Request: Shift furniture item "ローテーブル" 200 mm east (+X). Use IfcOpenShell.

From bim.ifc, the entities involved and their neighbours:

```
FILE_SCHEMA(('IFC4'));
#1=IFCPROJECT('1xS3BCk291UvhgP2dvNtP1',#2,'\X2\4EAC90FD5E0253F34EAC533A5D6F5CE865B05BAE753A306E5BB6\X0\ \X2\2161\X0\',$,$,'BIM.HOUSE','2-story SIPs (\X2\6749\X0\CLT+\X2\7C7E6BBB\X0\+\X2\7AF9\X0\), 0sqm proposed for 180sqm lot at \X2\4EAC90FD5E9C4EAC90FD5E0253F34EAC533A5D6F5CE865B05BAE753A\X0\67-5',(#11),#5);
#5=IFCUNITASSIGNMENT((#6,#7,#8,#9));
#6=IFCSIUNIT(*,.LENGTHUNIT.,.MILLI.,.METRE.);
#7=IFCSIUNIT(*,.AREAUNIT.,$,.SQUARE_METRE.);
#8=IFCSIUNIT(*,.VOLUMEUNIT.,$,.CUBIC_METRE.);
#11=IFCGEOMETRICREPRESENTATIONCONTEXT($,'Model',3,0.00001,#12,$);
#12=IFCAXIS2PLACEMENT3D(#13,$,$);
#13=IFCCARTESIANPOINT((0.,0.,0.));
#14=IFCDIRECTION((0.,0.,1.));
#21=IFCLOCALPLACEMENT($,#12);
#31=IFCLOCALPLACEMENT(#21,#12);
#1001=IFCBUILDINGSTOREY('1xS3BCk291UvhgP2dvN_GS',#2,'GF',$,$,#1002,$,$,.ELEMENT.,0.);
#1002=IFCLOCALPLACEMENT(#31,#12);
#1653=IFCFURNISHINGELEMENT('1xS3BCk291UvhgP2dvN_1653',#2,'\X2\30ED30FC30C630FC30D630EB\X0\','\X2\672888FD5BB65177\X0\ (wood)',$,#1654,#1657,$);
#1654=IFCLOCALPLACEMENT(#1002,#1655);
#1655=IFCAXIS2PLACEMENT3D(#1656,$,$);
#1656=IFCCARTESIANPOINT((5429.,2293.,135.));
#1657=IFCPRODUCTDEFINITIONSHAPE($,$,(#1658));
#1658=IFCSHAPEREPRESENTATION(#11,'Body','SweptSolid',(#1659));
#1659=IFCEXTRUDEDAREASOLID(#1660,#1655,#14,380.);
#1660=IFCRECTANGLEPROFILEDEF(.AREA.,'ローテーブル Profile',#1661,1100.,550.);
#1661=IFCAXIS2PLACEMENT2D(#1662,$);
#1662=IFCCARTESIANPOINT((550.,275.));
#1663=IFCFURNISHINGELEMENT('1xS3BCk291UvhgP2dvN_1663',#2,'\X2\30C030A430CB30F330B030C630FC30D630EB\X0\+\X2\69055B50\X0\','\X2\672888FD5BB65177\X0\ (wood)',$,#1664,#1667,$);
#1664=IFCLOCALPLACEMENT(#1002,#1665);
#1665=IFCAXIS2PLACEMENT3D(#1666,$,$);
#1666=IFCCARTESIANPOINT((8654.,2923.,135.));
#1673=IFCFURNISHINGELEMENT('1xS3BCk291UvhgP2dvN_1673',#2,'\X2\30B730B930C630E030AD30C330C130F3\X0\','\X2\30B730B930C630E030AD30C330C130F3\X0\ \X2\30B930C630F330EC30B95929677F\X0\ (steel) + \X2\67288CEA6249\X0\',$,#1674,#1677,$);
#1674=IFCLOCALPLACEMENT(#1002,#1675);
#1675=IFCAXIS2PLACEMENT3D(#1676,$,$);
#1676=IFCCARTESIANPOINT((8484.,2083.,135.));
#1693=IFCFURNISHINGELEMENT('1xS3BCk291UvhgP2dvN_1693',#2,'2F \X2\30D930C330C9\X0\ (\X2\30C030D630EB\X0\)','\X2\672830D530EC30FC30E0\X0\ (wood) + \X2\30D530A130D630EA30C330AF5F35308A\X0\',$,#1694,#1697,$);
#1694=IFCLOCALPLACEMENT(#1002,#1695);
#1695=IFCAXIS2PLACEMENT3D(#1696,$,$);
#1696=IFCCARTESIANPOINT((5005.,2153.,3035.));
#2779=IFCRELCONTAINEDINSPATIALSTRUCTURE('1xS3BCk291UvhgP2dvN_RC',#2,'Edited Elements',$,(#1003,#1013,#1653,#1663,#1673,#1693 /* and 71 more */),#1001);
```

```python
import ifcopenshell
import ifcopenshell.api.geometry
import ifcopenshell.util.placement
import ifcopenshell.util.unit

model = ifcopenshell.open("bim.ifc")
unit_scale = ifcopenshell.util.unit.calculate_unit_scale(model)

item = model.by_guid("1xS3BCk291UvhgP2dvN_1653")
matrix = ifcopenshell.util.placement.get_local_placement(item.ObjectPlacement)
matrix[0, 3] += 0.2 / unit_scale
ifcopenshell.api.geometry.edit_object_placement(model, product=item, matrix=matrix, is_si=False)

print(ifcopenshell.util.placement.get_local_placement(item.ObjectPlacement).round(3) + 0.0)

model.write("bim_rev.ifc")
```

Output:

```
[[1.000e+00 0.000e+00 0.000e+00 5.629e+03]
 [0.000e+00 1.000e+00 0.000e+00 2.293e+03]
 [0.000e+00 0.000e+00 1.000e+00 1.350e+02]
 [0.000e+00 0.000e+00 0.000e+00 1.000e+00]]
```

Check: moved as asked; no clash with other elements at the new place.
